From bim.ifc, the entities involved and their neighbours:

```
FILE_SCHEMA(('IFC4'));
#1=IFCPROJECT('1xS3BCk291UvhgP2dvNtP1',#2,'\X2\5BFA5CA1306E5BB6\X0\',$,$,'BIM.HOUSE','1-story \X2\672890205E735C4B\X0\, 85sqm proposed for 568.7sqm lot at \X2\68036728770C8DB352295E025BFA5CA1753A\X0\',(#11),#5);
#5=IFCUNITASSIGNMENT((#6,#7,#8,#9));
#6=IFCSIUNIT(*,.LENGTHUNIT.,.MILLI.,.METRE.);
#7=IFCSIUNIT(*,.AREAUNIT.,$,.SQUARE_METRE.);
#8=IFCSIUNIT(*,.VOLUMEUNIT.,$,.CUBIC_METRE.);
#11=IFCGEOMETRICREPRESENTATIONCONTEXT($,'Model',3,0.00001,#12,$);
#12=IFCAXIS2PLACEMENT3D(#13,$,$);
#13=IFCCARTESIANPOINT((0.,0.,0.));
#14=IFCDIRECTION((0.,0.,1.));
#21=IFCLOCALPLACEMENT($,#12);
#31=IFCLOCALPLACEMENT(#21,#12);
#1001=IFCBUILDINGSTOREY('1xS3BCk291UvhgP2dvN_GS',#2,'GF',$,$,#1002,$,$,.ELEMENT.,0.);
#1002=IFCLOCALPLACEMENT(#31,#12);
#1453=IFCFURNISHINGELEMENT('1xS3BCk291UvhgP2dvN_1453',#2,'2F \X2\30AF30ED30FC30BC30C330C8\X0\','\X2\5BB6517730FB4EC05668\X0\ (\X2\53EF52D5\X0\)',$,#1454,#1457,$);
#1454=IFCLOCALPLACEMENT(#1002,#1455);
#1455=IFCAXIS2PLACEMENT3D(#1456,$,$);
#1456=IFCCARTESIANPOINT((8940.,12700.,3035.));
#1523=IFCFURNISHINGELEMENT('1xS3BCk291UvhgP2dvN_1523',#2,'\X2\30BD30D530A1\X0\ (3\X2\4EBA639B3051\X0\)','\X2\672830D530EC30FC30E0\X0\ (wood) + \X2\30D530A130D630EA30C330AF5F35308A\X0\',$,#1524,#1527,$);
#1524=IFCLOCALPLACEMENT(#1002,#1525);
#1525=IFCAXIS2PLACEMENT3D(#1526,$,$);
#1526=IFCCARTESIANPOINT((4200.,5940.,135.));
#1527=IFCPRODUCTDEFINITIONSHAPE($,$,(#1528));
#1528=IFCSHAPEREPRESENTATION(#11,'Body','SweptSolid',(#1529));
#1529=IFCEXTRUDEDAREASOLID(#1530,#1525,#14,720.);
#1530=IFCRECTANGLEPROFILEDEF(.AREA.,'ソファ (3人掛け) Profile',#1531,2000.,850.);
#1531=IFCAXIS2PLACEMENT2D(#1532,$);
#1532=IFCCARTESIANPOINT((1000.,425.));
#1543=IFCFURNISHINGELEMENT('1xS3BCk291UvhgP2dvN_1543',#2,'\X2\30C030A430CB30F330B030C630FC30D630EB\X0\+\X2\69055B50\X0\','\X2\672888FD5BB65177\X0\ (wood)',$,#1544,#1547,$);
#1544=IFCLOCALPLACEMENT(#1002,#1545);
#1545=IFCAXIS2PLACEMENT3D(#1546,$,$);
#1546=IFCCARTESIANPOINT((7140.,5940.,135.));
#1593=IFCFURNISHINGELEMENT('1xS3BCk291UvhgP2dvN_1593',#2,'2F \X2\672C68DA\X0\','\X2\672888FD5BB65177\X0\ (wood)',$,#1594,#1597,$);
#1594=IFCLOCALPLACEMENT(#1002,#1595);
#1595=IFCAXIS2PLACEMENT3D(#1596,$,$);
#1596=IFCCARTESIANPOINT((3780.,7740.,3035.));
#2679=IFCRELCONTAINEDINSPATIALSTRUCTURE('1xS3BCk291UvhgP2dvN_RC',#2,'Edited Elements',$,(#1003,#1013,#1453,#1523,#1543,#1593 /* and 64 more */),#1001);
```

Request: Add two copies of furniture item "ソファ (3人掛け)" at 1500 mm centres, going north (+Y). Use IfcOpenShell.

```python
import numpy as np
import ifcopenshell
import ifcopenshell.api.geometry
import ifcopenshell.api.root
import ifcopenshell.util.element
import ifcopenshell.util.placement
import ifcopenshell.util.unit

model = ifcopenshell.open("bim.ifc")
unit_scale = ifcopenshell.util.unit.calculate_unit_scale(model)


def reuse_history(source, copy):
    """copy_class also copies each property set's owner history, people and application; keep the originals."""
    for rel in copy.IsDefinedBy:
        if rel.is_a("IfcRelDefinesByProperties") and (history := rel.RelatingPropertyDefinition.OwnerHistory):
            rel.RelatingPropertyDefinition.OwnerHistory = source.OwnerHistory
            ifcopenshell.util.element.remove_deep2(model, history)


source = model.by_guid("1xS3BCk291UvhgP2dvN_1523")
base = ifcopenshell.util.placement.get_local_placement(source.ObjectPlacement)
step = np.array([0.0, 1.0, 0.0]) * 1.5 / unit_scale

for i in range(1, 3):
    copy = ifcopenshell.api.root.copy_class(model, product=source)
    copy.Representation = ifcopenshell.util.element.copy_deep(
        model, source.Representation, exclude=["IfcGeometricRepresentationContext", "IfcRepresentationMap"]
    )
    reuse_history(source, copy)
    matrix = base.copy()
    matrix[:3, 3] += i * step
    print("added at", matrix[:3, 3].round(3) + 0.0)
    ifcopenshell.api.geometry.edit_object_placement(model, product=copy, matrix=matrix, is_si=False)

model.write("bim_edited.ifc")
```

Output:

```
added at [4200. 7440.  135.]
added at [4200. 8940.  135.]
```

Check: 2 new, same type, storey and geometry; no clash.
